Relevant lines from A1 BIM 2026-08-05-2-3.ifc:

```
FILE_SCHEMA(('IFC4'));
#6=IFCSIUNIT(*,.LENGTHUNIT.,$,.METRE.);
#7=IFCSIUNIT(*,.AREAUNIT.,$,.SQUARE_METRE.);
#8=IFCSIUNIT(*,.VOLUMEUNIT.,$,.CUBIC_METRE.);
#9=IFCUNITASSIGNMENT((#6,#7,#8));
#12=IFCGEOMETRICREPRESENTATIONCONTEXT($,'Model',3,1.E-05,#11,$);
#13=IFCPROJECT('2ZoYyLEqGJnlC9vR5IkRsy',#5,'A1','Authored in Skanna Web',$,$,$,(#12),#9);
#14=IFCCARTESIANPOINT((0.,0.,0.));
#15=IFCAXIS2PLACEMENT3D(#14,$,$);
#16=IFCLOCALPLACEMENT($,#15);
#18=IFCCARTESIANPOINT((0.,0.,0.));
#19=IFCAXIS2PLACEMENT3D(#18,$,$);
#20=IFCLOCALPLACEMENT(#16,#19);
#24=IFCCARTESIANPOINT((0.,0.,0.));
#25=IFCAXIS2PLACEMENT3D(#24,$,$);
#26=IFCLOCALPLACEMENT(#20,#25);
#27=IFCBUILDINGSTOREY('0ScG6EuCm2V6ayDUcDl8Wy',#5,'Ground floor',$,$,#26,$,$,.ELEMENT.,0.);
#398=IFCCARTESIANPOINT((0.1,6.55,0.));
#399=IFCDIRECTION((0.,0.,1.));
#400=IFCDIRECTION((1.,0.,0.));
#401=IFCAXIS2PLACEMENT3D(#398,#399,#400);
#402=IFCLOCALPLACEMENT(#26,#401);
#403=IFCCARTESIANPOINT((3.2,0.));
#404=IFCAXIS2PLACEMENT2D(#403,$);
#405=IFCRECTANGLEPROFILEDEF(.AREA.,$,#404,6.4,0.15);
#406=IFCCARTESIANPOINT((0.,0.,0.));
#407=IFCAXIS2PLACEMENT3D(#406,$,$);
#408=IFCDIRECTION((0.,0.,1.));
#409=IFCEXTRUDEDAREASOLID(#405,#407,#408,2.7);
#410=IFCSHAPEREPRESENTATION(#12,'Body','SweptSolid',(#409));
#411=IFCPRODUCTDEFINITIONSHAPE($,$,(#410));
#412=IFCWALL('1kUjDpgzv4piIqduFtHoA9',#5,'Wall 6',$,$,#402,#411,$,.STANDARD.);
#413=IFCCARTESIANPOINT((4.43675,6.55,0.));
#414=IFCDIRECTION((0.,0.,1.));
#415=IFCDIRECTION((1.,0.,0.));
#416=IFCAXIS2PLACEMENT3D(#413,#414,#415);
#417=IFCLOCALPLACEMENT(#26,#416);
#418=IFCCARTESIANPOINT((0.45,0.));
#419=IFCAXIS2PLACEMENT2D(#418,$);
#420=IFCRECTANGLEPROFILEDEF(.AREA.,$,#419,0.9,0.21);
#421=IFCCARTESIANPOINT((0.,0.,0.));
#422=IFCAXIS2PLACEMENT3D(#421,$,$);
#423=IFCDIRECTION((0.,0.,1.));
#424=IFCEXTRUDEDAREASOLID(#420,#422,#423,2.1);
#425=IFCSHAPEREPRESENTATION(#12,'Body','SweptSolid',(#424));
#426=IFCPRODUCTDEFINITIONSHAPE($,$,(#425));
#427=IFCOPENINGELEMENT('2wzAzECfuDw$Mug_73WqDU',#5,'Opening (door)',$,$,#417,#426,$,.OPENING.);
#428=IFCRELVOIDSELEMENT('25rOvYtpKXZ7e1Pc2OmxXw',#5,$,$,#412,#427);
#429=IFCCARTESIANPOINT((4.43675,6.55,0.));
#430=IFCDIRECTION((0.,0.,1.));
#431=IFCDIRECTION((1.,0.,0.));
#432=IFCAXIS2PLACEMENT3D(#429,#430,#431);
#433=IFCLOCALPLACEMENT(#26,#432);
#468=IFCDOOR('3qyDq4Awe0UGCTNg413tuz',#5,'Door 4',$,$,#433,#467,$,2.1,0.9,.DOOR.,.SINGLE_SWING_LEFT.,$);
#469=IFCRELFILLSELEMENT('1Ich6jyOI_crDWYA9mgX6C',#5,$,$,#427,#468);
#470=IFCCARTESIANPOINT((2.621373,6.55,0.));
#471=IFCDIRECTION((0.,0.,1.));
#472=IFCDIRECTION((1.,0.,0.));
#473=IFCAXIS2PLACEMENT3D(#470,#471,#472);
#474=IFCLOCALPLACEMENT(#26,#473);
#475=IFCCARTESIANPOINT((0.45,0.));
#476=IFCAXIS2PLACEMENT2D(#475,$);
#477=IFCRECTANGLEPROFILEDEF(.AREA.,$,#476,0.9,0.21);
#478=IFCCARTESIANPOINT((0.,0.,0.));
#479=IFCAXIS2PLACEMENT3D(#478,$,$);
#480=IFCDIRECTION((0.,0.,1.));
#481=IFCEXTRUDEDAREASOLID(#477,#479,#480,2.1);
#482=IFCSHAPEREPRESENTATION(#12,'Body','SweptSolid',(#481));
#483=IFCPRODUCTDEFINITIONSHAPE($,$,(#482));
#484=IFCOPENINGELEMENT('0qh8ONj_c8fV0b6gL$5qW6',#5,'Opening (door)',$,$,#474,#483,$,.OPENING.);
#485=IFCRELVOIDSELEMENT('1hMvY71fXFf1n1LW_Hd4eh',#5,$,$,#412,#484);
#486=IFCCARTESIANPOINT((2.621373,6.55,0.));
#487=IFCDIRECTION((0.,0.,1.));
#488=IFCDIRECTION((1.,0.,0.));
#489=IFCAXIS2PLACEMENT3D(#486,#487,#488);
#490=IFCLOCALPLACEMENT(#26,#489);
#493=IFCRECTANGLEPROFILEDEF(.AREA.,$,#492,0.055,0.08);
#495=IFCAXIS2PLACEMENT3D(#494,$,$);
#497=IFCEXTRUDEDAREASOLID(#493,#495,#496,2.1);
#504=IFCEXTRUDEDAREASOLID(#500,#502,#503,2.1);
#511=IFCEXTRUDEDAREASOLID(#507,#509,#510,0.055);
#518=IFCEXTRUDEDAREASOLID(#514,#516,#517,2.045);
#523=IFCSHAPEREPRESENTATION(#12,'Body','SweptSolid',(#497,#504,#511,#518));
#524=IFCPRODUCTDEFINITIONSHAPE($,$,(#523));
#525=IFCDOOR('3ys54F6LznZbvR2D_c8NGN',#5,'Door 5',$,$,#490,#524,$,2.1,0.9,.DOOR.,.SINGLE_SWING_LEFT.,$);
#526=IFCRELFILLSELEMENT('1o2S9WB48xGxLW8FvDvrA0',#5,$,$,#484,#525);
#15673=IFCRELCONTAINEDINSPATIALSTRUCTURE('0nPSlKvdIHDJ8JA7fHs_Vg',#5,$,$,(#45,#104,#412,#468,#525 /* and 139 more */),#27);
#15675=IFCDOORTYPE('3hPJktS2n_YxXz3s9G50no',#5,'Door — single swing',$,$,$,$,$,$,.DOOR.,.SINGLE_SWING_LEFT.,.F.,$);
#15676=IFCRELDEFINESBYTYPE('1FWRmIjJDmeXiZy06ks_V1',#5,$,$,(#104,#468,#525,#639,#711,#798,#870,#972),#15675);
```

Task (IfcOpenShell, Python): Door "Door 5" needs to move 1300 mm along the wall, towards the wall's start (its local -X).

```python
import ifcopenshell
import ifcopenshell.api.geometry
import ifcopenshell.util.placement
import ifcopenshell.util.unit

model = ifcopenshell.open("A1 BIM 2026-08-05-2-3.ifc")
unit_scale = ifcopenshell.util.unit.calculate_unit_scale(model)

door = model.by_guid("3ys54F6LznZbvR2D_c8NGN")
opening = door.FillsVoids[0].RelatingOpeningElement
wall = opening.VoidsElements[0].RelatingBuildingElement

wall_matrix = ifcopenshell.util.placement.get_local_placement(wall.ObjectPlacement)
shift = wall_matrix[:3, 0] * -1.3 / unit_scale
before = ifcopenshell.util.placement.get_local_placement(door.ObjectPlacement)[:3, 3].copy()

# The door is not placed relative to its opening, so move both.
for product in (opening, door):
    matrix = ifcopenshell.util.placement.get_local_placement(product.ObjectPlacement)
    matrix[:3, 3] += shift
    ifcopenshell.api.geometry.edit_object_placement(model, product=product, matrix=matrix, is_si=False)

after = ifcopenshell.util.placement.get_local_placement(door.ObjectPlacement)[:3, 3]
print("door moved by", (after - before).round(3) + 0.0)

model.write("A1 BIM 2026-08-05-2-3_rev.ifc")
```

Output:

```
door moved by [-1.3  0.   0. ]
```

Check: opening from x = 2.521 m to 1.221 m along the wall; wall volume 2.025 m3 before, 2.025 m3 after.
